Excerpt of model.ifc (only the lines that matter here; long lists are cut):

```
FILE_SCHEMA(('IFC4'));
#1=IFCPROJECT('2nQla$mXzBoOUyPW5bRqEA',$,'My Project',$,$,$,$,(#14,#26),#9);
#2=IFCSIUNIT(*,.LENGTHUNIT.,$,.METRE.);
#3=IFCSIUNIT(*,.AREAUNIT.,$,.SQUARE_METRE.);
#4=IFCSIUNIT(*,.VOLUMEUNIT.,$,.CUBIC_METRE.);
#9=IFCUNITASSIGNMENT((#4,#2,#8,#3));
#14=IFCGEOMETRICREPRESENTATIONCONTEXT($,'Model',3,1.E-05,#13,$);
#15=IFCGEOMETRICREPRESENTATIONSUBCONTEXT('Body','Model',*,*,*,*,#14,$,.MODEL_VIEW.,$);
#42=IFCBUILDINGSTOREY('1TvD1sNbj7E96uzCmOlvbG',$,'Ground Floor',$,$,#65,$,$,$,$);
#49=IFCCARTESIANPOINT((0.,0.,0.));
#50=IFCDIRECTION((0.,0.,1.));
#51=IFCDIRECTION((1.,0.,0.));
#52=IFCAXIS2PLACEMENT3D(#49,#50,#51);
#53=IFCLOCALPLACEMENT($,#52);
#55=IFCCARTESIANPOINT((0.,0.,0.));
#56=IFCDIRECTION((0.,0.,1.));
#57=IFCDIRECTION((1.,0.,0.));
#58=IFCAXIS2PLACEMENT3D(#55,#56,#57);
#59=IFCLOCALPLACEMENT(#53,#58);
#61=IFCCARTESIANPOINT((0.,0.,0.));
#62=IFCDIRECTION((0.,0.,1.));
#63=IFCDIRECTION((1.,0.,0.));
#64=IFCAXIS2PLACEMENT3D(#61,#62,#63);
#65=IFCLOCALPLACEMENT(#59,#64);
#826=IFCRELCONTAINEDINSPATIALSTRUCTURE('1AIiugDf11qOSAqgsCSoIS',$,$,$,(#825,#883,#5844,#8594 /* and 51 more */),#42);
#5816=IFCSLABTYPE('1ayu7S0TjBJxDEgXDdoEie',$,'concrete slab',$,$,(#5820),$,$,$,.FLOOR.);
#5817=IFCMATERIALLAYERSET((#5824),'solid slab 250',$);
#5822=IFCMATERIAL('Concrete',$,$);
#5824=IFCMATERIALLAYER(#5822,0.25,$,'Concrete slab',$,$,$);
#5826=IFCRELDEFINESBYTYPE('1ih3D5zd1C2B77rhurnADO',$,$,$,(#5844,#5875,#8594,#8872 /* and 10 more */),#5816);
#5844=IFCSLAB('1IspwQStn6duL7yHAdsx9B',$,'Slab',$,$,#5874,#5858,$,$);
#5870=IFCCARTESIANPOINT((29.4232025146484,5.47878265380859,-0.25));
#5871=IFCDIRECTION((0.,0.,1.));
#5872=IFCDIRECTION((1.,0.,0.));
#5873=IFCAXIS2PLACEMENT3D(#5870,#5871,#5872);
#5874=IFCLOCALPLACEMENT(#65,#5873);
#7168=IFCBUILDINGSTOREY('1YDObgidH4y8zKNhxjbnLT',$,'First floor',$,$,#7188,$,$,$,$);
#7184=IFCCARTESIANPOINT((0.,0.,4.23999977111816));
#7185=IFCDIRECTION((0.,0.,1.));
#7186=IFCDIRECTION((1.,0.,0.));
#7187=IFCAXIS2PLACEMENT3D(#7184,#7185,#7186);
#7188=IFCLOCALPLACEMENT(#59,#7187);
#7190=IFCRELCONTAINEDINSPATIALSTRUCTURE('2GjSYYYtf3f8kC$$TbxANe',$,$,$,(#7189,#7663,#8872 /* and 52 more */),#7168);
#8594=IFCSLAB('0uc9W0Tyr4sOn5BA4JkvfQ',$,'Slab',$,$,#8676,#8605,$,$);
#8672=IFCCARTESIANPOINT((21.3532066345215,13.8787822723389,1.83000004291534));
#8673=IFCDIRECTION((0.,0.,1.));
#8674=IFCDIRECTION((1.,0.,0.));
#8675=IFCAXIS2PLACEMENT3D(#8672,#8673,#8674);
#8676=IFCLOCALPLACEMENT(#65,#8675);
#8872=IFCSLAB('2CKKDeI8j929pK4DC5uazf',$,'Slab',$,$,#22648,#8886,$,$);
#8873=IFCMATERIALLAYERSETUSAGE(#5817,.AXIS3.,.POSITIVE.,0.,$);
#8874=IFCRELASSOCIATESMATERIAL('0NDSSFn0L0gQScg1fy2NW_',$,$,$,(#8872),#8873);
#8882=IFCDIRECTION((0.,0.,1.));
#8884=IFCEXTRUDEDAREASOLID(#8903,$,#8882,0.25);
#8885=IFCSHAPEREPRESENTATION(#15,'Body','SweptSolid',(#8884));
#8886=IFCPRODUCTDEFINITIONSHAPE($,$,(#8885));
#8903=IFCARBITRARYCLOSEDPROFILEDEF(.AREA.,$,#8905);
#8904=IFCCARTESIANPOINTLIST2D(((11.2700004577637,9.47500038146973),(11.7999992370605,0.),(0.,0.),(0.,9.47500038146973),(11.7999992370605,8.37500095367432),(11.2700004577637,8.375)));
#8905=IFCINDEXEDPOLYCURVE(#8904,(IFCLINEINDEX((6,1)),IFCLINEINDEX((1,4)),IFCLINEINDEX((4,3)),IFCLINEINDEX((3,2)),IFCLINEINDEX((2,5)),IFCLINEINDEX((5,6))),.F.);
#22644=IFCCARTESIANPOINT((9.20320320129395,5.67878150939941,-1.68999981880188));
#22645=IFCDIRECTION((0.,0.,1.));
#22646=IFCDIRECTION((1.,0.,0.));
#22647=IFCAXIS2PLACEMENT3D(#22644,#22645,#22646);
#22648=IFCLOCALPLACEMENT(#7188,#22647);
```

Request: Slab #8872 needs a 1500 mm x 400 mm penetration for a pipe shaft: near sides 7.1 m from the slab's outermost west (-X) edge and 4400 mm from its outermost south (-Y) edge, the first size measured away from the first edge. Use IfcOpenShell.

```python
import numpy as np
import ifcopenshell
import ifcopenshell.api.feature
import ifcopenshell.api.geometry
import ifcopenshell.api.root
import ifcopenshell.geom
import ifcopenshell.util.placement
import ifcopenshell.util.representation
import ifcopenshell.util.shape
import ifcopenshell.util.unit

model = ifcopenshell.open("model.ifc")
unit_scale = ifcopenshell.util.unit.calculate_unit_scale(model)
settings = ifcopenshell.geom.settings()


def volume(element):
    """Net volume in cubic metres, openings subtracted."""
    shape = ifcopenshell.geom.create_shape(settings, element)
    return ifcopenshell.util.shape.get_volume(shape.geometry)


slab = model.by_guid("2CKKDeI8j929pK4DC5uazf")
before = volume(slab)

# Extent in the slab's own axes, in metres. The edges named are its -X and -Y sides.
slab_shape = ifcopenshell.geom.create_shape(settings, slab)
vertices = ifcopenshell.util.shape.get_vertices(slab_shape.geometry)
x_min, y_min, bottom = vertices.min(axis=0)
top = vertices[:, 2].max()

opening = ifcopenshell.api.root.create_entity(model, ifc_class="IfcOpeningElement", name="Pipe shaft opening", predefined_type="OPENING")
context = ifcopenshell.util.representation.get_context(model, "Model", "Body", "MODEL_VIEW")
width, depth = 1.5, 0.4
outline = [(0.0, 0.0), (width, 0.0), (width, depth), (0.0, depth), (0.0, 0.0)]
# Overshoot both faces by 50 mm so the cut is clean.
shape = ifcopenshell.api.geometry.add_slab_representation(
    model, context=context, depth=top - bottom + 0.1, polyline=outline
)
ifcopenshell.api.geometry.assign_representation(model, product=opening, representation=shape)

matrix = ifcopenshell.util.placement.get_local_placement(slab.ObjectPlacement)
matrix[:, 3] = matrix @ np.append(np.array([x_min + 7.1, y_min + 4.4, bottom - 0.05]) / unit_scale, 1.0)
ifcopenshell.api.geometry.edit_object_placement(model, product=opening, matrix=matrix, is_si=False)
ifcopenshell.api.feature.add_feature(model, feature=opening, element=slab)

after = volume(slab)

print(f"slab volume {before:.3f} -> {after:.3f} m3")

model.write("model_updated.ifc")
```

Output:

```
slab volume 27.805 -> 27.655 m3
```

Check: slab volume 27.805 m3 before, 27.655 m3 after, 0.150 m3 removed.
